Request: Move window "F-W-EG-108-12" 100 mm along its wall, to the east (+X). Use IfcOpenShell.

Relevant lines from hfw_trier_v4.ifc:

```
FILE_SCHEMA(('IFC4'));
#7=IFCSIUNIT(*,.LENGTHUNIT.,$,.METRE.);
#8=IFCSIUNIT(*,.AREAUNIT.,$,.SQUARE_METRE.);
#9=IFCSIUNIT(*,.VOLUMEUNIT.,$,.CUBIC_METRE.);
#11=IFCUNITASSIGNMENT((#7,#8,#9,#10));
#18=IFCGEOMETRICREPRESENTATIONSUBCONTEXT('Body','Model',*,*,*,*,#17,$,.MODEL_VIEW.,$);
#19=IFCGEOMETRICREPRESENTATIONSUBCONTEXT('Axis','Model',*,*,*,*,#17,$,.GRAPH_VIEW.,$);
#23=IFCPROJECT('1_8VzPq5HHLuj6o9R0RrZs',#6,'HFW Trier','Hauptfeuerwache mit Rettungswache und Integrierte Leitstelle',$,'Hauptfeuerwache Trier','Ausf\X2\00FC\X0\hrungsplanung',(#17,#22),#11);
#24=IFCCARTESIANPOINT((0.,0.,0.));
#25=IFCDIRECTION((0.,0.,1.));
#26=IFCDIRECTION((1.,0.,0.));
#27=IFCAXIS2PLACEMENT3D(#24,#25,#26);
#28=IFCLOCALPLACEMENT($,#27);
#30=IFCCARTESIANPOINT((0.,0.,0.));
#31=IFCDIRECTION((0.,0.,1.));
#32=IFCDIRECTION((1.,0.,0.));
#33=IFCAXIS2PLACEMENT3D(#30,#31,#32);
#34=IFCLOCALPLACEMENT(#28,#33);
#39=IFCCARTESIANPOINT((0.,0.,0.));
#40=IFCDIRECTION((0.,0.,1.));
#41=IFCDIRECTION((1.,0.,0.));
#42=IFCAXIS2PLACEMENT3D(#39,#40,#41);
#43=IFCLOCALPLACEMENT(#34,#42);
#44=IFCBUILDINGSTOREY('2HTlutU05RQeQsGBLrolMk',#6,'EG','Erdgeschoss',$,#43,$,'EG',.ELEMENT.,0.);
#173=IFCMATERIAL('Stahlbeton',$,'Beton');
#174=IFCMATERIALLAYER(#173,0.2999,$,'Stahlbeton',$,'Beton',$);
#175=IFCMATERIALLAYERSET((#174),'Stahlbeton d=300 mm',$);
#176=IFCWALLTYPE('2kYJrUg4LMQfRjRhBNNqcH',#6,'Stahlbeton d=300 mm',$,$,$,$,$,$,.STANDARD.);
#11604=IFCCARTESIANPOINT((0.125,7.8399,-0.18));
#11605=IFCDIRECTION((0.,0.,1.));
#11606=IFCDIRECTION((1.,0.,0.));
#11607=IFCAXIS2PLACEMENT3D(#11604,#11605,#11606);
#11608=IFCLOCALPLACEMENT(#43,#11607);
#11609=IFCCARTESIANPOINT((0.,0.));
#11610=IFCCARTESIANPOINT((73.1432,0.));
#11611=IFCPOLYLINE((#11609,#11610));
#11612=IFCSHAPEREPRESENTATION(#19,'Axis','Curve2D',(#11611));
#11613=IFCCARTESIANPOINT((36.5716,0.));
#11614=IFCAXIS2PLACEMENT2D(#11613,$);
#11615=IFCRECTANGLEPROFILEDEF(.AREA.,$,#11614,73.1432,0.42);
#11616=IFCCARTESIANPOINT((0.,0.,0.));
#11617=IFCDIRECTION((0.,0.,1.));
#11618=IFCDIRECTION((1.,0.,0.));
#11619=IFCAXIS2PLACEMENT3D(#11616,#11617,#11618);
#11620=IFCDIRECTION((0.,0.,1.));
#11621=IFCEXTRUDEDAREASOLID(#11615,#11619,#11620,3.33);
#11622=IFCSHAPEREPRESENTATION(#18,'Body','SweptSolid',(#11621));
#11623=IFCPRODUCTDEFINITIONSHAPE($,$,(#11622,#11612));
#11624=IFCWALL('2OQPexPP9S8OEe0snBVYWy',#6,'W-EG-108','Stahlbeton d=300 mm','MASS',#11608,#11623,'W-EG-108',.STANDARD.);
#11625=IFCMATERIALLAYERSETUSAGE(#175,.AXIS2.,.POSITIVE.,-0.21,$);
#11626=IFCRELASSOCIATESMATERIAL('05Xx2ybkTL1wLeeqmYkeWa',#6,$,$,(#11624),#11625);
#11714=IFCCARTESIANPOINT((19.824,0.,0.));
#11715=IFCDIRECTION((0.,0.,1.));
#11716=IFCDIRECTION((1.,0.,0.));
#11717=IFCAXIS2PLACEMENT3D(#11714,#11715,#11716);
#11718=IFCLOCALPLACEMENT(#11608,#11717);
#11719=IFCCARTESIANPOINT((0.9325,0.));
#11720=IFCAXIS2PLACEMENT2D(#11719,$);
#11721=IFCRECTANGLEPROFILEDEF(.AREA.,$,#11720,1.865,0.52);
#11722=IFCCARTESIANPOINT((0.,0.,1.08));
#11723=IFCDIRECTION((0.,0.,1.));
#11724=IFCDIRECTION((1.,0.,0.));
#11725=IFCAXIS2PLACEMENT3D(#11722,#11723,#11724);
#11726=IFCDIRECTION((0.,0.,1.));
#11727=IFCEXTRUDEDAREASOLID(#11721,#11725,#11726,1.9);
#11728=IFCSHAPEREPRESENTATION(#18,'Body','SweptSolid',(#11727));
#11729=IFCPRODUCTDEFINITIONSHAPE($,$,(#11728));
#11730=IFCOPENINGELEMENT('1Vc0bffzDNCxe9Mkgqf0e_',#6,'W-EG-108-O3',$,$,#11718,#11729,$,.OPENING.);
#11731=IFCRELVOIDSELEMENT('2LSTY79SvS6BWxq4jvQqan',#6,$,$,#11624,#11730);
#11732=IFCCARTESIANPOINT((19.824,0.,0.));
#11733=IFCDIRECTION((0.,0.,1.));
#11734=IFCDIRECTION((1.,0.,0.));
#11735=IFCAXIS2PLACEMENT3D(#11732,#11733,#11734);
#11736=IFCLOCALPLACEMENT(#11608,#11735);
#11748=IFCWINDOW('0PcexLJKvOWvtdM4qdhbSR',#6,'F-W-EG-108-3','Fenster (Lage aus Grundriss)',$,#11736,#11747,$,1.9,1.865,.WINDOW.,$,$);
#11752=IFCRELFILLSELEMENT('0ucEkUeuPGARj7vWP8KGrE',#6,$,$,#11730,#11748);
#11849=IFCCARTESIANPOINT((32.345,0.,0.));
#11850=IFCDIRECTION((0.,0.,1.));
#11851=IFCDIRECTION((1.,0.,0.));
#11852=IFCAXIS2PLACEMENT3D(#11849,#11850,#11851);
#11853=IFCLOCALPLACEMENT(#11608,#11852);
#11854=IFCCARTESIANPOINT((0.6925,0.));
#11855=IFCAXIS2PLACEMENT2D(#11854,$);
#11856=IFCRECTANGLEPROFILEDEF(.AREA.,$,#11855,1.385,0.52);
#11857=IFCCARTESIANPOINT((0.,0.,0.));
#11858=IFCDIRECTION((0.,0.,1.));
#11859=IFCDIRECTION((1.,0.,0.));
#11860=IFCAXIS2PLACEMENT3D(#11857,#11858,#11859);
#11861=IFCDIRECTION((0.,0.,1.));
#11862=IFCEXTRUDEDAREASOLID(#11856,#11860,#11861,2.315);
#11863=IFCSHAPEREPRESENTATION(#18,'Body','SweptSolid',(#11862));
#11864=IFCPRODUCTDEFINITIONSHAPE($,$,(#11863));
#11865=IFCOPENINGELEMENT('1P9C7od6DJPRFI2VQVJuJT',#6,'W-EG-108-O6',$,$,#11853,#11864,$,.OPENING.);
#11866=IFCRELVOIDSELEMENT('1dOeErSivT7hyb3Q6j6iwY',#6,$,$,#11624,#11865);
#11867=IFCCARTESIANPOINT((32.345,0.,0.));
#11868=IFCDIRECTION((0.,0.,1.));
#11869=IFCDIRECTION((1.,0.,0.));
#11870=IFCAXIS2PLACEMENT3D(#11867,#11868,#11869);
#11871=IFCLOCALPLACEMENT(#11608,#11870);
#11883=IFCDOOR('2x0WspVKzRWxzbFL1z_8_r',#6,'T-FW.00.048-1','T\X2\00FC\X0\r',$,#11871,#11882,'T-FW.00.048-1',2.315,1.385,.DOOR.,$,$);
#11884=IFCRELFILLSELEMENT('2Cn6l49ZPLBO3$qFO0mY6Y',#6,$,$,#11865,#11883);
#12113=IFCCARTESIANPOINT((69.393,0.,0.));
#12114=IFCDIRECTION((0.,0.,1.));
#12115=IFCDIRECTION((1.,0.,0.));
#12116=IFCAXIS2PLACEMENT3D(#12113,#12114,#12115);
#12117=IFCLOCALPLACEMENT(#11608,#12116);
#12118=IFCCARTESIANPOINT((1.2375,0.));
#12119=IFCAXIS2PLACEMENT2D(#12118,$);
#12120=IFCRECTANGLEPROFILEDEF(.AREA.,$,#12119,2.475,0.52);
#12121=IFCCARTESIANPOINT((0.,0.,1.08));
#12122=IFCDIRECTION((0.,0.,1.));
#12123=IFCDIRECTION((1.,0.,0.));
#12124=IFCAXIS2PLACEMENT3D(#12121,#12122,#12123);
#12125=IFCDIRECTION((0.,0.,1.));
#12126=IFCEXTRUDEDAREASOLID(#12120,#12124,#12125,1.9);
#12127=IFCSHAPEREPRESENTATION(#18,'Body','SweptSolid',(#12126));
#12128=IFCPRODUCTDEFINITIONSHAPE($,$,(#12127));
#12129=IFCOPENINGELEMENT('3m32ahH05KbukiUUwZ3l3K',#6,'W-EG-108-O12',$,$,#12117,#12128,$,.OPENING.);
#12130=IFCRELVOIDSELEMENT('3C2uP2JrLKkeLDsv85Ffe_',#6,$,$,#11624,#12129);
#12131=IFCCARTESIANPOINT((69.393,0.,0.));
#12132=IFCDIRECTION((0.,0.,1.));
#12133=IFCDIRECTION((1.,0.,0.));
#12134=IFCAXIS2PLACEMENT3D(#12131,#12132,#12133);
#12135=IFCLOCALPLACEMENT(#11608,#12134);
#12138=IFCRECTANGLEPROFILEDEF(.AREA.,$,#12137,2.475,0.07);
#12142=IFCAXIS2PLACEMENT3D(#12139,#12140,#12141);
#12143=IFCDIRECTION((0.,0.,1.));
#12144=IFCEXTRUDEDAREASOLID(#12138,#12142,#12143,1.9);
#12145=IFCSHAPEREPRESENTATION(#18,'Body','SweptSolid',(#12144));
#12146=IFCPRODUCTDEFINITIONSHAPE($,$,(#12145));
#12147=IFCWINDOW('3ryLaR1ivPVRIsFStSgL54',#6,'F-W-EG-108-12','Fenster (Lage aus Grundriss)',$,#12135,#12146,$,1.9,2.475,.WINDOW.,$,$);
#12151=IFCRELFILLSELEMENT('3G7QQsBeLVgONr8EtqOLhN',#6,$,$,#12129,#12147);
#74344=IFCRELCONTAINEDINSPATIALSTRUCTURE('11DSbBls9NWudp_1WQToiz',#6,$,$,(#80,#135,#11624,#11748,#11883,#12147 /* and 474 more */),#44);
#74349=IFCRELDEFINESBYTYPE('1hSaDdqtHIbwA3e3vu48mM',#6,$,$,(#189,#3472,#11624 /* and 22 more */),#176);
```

```python
import ifcopenshell
import ifcopenshell.api.geometry
import ifcopenshell.util.placement

model = ifcopenshell.open("hfw_trier_v4.ifc")

window = model.by_guid("3ryLaR1ivPVRIsFStSgL54")
opening = window.FillsVoids[0].RelatingOpeningElement
wall = opening.VoidsElements[0].RelatingBuildingElement

wall_matrix = ifcopenshell.util.placement.get_local_placement(wall.ObjectPlacement)
shift = wall_matrix[:3, 0] * 0.1
before = ifcopenshell.util.placement.get_local_placement(window.ObjectPlacement)[:3, 3].copy()

# The window is not placed relative to its opening, so move both.
for product in (opening, window):
    matrix = ifcopenshell.util.placement.get_local_placement(product.ObjectPlacement)
    matrix[:3, 3] += shift
    ifcopenshell.api.geometry.edit_object_placement(model, product=product, matrix=matrix, is_si=False)

after = ifcopenshell.util.placement.get_local_placement(window.ObjectPlacement)[:3, 3]
print("window moved by", (after - before).round(3) + 0.0)

model.write("hfw_trier_v4_v2.ifc")
```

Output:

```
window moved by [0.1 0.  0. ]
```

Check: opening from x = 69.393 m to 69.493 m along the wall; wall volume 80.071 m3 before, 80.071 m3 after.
